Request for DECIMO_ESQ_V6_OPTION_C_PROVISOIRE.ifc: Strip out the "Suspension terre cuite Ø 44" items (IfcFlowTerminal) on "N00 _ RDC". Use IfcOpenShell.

First a look at what the model holds.

```python
import ifcopenshell
import ifcopenshell.util.element

model = ifcopenshell.open("DECIMO_ESQ_V6_OPTION_C_PROVISOIRE.ifc")
print(model.schema)
storey = next(s for s in model.by_type("IfcBuildingStorey") if s.Name == "N00 _ RDC")
terminals = [e for e in ifcopenshell.util.element.get_decomposition(storey) if e.is_a("IfcFlowTerminal")]
seen = {}
for e in terminals:
    element_type = ifcopenshell.util.element.get_type(e)
    name = element_type.Name if element_type not in (None, e) else None
    seen[name] = seen.get(name, 0) + 1
for name, count in sorted(seen.items(), key=str):
    print(count, "x", name)
```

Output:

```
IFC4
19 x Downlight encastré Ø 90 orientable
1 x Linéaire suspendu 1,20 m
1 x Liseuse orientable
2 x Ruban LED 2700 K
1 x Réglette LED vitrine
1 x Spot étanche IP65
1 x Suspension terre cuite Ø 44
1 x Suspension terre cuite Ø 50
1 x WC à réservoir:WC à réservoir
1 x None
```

```python
import ifcopenshell
import ifcopenshell.api.root
import ifcopenshell.util.element

model = ifcopenshell.open("DECIMO_ESQ_V6_OPTION_C_PROVISOIRE.ifc")

storey = next(s for s in model.by_type("IfcBuildingStorey") if s.Name == "N00 _ RDC")
terminals = [e for e in ifcopenshell.util.element.get_decomposition(storey) if e.is_a("IfcFlowTerminal")]
targets = [e for e in terminals if (t := ifcopenshell.util.element.get_type(e)) not in (None, e) and t.Name == "Suspension terre cuite Ø 44"]

for e in targets:
    ifcopenshell.api.root.remove_product(model, product=e)
print(len(targets), "removed")

model.write("DECIMO_ESQ_V6_OPTION_C_PROVISOIRE_rev.ifc")
```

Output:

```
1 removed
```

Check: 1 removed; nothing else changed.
